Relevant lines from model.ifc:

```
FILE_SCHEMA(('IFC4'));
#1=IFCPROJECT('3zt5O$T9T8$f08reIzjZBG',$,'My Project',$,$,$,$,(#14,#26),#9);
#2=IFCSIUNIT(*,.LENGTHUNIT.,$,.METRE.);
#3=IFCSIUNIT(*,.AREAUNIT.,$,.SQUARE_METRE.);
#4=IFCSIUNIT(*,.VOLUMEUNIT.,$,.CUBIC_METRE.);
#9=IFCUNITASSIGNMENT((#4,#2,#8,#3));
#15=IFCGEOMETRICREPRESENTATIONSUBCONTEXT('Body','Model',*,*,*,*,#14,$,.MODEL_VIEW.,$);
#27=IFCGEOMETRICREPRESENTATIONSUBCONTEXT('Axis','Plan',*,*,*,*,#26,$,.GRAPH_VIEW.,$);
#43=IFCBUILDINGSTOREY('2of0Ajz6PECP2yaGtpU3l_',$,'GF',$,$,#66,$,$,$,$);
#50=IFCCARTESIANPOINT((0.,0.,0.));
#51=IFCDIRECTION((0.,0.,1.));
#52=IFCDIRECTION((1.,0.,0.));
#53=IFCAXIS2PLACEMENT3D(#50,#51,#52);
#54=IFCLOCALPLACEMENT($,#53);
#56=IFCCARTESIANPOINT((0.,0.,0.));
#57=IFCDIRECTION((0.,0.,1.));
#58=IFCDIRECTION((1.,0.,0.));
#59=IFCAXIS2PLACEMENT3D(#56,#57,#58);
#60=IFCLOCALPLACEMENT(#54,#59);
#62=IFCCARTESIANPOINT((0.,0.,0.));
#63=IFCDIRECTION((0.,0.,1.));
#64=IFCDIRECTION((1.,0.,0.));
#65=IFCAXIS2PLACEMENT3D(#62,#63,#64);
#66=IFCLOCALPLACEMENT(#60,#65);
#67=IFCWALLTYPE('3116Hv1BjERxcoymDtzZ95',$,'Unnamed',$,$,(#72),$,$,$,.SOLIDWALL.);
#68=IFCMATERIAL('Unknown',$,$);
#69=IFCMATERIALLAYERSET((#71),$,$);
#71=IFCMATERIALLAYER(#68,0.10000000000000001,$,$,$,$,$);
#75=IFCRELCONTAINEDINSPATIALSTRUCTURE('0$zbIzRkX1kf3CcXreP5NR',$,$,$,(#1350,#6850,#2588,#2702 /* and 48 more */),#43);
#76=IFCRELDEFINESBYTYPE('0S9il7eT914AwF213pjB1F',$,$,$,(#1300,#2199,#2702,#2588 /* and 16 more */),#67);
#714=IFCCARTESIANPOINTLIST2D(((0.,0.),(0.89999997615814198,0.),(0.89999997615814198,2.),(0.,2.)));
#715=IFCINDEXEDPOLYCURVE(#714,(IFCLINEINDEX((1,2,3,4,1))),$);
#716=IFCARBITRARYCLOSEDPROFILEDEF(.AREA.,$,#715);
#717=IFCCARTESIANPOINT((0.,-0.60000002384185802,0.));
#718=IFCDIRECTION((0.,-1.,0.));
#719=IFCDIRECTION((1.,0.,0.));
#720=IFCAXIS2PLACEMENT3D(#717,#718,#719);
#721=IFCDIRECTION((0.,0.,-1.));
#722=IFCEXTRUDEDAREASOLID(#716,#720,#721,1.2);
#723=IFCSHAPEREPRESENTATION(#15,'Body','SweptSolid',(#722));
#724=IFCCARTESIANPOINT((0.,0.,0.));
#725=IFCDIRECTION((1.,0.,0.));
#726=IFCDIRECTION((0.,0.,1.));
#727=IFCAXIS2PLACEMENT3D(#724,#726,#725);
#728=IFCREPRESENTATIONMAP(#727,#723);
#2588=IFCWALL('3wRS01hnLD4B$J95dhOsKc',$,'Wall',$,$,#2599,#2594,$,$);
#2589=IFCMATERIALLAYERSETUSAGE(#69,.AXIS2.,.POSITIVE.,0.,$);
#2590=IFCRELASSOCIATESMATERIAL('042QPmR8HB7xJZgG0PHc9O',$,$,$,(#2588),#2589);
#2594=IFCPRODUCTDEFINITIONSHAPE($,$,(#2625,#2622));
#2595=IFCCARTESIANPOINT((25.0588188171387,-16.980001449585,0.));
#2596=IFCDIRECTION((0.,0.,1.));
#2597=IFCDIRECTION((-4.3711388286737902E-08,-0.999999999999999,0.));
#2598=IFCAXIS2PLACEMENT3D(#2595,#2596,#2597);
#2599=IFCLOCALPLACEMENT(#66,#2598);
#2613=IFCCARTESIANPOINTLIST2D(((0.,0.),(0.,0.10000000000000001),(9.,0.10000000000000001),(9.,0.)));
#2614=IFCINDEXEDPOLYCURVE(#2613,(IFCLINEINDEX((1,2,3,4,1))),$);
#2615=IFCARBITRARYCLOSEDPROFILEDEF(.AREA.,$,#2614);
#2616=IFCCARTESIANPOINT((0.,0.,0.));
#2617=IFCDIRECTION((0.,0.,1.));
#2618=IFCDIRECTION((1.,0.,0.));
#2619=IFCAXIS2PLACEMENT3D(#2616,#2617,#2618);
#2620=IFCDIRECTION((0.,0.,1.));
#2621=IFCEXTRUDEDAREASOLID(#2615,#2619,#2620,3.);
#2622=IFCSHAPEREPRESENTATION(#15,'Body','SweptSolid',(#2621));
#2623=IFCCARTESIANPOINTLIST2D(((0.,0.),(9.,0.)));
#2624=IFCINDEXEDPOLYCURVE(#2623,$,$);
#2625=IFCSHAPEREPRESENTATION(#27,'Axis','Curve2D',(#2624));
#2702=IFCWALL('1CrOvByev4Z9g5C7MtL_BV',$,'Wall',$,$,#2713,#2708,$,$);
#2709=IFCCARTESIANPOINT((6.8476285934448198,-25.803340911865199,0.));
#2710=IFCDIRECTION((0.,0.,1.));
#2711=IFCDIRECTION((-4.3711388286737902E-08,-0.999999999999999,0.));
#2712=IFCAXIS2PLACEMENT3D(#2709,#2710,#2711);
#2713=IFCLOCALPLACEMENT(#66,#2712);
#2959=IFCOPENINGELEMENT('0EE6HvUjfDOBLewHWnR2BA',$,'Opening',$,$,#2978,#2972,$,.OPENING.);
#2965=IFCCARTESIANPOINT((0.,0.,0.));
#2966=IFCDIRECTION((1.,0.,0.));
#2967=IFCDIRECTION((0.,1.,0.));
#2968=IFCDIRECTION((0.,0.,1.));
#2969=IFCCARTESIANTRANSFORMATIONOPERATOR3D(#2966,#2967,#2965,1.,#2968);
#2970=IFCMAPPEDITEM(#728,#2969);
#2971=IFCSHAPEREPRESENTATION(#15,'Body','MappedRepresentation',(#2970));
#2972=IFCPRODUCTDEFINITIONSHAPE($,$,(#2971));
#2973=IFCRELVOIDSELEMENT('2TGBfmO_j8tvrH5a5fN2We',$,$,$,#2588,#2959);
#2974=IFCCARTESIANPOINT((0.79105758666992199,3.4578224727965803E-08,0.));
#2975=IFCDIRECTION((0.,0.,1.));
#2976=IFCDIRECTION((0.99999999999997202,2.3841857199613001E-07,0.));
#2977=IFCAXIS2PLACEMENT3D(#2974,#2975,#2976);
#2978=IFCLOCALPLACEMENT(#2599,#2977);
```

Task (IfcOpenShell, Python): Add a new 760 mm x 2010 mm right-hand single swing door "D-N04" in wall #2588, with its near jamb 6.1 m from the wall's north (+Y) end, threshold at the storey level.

```python
import numpy as np
import ifcopenshell
import ifcopenshell.api.feature
import ifcopenshell.api.geometry
import ifcopenshell.api.root
import ifcopenshell.api.spatial
import ifcopenshell.geom
import ifcopenshell.util.element
import ifcopenshell.util.placement
import ifcopenshell.util.representation
import ifcopenshell.util.shape
import ifcopenshell.util.unit

model = ifcopenshell.open("model.ifc")
unit_scale = ifcopenshell.util.unit.calculate_unit_scale(model)
settings = ifcopenshell.geom.settings()


def volume(element):
    """Net volume in cubic metres, openings subtracted."""
    shape = ifcopenshell.geom.create_shape(settings, element)
    return ifcopenshell.util.shape.get_volume(shape.geometry)


wall = model.by_guid("3wRS01hnLD4B$J95dhOsKc")
storey = ifcopenshell.util.element.get_container(wall, ifc_class="IfcBuildingStorey")
context = ifcopenshell.util.representation.get_context(model, "Model", "Body", "MODEL_VIEW")
before = volume(wall)

width, height, from_end, sill = 0.76, 2.01, 6.1, 0.0  # metres

# The wall runs along its own X axis, and the end named is its -X end.
wall_shape = ifcopenshell.geom.create_shape(settings, wall)
x, y, z = ifcopenshell.util.shape.get_vertices(wall_shape.geometry).T
start = x.min() + from_end
face, thickness = float(y.min()), float(y.max() - y.min())
wall_matrix = ifcopenshell.util.placement.get_local_placement(wall.ObjectPlacement)
level = ifcopenshell.util.placement.get_local_placement(storey.ObjectPlacement)[2, 3]


def in_wall(x, y):
    """Placement at x, y metres in the wall's axes, at sill height."""
    matrix = wall_matrix.copy()
    matrix[:, 3] = wall_matrix @ np.array([x / unit_scale, y / unit_scale, 0.0, 1.0])
    matrix[2, 3] = level + sill / unit_scale
    return matrix


# Opening: a box that overshoots both wall faces by 50 mm.
opening = ifcopenshell.api.root.create_entity(model, ifc_class="IfcOpeningElement", predefined_type="OPENING")
box = ifcopenshell.api.geometry.add_wall_representation(
    model, context=context, length=width, height=height, thickness=thickness + 0.1
)
ifcopenshell.api.geometry.assign_representation(model, product=opening, representation=box)
ifcopenshell.api.geometry.edit_object_placement(model, product=opening, matrix=in_wall(start, face - 0.05), is_si=False)
ifcopenshell.api.feature.add_feature(model, feature=opening, element=wall)

door = ifcopenshell.api.root.create_entity(model, ifc_class="IfcDoor", name="D-N04", predefined_type="DOOR")
door.OverallWidth, door.OverallHeight = width / unit_scale, height / unit_scale
door.OperationType = "SINGLE_SWING_RIGHT"
body = ifcopenshell.api.geometry.add_door_representation(
    model,
    context=context,
    overall_width=door.OverallWidth,
    overall_height=door.OverallHeight,
    operation_type="SINGLE_SWING_RIGHT",
    lining_properties={"LiningDepth": thickness / unit_scale, "ThresholdDepth": thickness / unit_scale},
)
ifcopenshell.api.geometry.assign_representation(model, product=door, representation=body)
ifcopenshell.api.spatial.assign_container(model, products=[door], relating_structure=storey)
ifcopenshell.api.feature.add_filling(model, opening=opening, element=door)

# The lining spans the wall, so the door starts at the wall face.
ifcopenshell.api.geometry.edit_object_placement(model, product=door, matrix=in_wall(start, face), is_si=False)

after = volume(wall)

print(f"wall volume {before:.3f} -> {after:.3f} m3")

model.write("model_updated.ifc")
```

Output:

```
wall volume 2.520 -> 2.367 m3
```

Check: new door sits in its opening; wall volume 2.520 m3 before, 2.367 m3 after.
